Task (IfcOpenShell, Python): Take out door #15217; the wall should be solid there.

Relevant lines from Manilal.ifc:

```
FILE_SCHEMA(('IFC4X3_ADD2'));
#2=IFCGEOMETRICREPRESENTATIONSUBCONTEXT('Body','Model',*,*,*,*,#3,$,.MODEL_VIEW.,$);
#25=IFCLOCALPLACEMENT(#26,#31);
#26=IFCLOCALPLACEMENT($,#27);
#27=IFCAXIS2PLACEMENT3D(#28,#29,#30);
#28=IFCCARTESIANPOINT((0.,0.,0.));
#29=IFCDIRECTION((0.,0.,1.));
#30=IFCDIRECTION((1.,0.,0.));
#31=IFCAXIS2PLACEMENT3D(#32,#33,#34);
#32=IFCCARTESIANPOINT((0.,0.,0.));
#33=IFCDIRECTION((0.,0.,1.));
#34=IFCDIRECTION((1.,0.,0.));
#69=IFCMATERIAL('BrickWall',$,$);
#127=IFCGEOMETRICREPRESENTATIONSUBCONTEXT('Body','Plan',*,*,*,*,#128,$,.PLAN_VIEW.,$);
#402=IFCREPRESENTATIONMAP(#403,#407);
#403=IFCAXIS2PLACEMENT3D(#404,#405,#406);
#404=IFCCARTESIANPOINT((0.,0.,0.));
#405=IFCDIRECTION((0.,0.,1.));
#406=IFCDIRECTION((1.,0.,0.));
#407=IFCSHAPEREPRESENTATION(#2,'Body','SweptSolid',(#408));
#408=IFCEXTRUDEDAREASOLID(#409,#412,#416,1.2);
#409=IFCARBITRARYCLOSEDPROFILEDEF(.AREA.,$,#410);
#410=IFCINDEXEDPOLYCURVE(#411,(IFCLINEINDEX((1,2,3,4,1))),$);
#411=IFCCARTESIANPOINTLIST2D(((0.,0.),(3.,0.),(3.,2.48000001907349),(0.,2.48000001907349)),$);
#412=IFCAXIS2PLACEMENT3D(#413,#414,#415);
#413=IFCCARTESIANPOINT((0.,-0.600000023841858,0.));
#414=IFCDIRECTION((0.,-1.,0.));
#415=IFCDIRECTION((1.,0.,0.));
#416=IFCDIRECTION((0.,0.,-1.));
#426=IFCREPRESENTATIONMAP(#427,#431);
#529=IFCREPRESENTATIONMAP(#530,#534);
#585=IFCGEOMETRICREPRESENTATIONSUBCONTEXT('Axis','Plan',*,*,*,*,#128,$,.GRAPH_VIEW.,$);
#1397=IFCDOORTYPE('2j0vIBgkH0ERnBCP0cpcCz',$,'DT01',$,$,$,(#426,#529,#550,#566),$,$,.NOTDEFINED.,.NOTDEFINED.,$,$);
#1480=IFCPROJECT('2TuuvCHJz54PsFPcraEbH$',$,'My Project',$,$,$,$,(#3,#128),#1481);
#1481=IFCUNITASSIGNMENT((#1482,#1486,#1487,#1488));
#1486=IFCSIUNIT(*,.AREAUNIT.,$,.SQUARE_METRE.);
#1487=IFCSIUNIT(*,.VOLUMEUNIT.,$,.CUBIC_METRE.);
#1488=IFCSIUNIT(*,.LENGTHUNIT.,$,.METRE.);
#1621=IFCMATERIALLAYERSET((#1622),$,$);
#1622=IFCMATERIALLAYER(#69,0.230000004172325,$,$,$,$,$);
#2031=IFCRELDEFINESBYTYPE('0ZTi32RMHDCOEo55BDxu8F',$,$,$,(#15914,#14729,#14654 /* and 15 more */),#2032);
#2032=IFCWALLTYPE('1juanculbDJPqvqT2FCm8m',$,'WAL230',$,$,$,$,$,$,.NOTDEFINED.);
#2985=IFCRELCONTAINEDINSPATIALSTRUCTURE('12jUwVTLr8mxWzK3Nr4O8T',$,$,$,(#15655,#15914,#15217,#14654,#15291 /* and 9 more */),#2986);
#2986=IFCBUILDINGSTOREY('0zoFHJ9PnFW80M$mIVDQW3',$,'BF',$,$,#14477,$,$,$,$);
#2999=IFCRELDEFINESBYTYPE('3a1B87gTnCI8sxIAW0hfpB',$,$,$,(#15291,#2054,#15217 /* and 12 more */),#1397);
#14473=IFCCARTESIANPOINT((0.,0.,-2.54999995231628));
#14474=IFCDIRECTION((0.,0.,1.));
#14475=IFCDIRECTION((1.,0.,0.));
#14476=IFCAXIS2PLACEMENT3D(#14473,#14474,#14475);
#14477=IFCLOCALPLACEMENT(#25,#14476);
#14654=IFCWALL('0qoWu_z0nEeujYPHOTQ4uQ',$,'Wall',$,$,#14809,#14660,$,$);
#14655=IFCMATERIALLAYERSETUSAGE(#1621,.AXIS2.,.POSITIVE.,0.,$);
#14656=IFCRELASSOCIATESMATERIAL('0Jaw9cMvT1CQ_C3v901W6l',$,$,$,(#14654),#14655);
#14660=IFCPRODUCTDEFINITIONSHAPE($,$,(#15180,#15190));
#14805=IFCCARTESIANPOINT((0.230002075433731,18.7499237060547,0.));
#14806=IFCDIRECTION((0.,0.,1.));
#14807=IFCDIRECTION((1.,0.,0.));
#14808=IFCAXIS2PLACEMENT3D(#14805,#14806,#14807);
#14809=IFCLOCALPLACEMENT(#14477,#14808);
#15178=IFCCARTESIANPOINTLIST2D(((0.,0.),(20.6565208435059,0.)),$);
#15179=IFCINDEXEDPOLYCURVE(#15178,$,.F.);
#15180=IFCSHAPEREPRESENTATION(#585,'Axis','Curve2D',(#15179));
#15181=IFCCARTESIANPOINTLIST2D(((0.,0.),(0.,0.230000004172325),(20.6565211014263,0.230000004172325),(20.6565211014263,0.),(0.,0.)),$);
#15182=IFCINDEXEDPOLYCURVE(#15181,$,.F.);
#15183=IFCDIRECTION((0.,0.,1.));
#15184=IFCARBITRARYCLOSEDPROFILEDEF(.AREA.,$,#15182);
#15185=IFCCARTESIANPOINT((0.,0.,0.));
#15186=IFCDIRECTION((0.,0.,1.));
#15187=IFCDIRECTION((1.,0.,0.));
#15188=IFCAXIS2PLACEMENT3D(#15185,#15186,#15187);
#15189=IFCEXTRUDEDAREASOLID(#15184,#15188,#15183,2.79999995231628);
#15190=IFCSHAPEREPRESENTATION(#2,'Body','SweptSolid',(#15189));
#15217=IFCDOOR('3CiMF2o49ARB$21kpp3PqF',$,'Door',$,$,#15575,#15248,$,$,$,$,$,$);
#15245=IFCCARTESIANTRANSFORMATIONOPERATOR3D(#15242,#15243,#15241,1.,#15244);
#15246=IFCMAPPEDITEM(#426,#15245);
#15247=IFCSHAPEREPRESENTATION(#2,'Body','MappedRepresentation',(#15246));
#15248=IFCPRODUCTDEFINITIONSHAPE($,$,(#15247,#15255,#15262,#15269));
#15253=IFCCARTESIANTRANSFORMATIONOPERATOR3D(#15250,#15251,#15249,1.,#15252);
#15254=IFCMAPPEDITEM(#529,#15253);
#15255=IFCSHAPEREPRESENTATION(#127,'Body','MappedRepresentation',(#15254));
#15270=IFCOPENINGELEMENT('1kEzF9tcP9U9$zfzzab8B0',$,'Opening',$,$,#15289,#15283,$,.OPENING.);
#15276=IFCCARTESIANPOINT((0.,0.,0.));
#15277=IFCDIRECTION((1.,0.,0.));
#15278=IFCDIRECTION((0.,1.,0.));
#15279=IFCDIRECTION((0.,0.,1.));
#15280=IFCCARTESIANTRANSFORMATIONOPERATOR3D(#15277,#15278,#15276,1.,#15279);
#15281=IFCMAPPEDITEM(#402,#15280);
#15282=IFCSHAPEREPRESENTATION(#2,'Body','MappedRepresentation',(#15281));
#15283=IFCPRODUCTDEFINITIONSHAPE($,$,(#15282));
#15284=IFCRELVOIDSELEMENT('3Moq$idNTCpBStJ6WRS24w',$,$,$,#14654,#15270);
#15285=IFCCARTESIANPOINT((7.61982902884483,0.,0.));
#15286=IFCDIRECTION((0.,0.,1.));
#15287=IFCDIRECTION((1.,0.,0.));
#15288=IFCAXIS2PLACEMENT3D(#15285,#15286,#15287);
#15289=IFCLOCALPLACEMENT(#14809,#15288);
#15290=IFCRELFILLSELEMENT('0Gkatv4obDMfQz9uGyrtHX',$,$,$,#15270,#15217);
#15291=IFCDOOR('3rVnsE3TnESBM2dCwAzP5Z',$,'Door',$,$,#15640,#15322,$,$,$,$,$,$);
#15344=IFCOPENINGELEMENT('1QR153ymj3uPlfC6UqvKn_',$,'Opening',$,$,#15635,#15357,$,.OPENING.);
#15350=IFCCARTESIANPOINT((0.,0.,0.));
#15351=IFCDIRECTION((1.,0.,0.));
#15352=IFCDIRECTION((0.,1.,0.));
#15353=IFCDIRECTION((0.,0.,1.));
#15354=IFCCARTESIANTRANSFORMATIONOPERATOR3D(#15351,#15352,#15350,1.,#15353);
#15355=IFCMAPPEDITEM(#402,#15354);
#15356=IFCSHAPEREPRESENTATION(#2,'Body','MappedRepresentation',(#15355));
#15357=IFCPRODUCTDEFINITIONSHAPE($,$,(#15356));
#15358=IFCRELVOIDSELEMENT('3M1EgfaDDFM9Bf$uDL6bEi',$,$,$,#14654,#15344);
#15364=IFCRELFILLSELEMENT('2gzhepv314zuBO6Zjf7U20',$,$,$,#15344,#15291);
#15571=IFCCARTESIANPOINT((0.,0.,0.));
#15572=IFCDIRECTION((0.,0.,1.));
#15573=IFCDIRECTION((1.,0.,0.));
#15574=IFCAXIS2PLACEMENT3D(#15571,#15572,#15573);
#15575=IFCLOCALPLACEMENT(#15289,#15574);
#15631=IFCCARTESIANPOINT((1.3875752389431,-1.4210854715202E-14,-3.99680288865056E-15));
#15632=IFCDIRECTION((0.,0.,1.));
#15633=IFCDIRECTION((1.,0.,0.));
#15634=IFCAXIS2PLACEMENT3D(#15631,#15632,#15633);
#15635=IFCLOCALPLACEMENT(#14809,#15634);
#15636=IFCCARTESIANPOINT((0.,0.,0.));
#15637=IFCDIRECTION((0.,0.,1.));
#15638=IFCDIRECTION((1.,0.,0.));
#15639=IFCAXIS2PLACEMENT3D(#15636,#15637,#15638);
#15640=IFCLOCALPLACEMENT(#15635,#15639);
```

```python
import ifcopenshell
import ifcopenshell.api.feature
import ifcopenshell.api.root
import ifcopenshell.geom
import ifcopenshell.util.shape

model = ifcopenshell.open("Manilal.ifc")
settings = ifcopenshell.geom.settings()


def volume(element):
    """Net volume in cubic metres, openings subtracted."""
    shape = ifcopenshell.geom.create_shape(settings, element)
    return ifcopenshell.util.shape.get_volume(shape.geometry)


door = model.by_guid("3CiMF2o49ARB$21kpp3PqF")
opening = door.FillsVoids[0].RelatingOpeningElement
wall = opening.VoidsElements[0].RelatingBuildingElement
before = volume(wall)

ifcopenshell.api.root.remove_product(model, product=door)
ifcopenshell.api.feature.remove_feature(model, feature=opening)

after = volume(wall)

print(f"wall volume {before:.3f} -> {after:.3f} m3")

model.write("Manilal_v2.ifc")
```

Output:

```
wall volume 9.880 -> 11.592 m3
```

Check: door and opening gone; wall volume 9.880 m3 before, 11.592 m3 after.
